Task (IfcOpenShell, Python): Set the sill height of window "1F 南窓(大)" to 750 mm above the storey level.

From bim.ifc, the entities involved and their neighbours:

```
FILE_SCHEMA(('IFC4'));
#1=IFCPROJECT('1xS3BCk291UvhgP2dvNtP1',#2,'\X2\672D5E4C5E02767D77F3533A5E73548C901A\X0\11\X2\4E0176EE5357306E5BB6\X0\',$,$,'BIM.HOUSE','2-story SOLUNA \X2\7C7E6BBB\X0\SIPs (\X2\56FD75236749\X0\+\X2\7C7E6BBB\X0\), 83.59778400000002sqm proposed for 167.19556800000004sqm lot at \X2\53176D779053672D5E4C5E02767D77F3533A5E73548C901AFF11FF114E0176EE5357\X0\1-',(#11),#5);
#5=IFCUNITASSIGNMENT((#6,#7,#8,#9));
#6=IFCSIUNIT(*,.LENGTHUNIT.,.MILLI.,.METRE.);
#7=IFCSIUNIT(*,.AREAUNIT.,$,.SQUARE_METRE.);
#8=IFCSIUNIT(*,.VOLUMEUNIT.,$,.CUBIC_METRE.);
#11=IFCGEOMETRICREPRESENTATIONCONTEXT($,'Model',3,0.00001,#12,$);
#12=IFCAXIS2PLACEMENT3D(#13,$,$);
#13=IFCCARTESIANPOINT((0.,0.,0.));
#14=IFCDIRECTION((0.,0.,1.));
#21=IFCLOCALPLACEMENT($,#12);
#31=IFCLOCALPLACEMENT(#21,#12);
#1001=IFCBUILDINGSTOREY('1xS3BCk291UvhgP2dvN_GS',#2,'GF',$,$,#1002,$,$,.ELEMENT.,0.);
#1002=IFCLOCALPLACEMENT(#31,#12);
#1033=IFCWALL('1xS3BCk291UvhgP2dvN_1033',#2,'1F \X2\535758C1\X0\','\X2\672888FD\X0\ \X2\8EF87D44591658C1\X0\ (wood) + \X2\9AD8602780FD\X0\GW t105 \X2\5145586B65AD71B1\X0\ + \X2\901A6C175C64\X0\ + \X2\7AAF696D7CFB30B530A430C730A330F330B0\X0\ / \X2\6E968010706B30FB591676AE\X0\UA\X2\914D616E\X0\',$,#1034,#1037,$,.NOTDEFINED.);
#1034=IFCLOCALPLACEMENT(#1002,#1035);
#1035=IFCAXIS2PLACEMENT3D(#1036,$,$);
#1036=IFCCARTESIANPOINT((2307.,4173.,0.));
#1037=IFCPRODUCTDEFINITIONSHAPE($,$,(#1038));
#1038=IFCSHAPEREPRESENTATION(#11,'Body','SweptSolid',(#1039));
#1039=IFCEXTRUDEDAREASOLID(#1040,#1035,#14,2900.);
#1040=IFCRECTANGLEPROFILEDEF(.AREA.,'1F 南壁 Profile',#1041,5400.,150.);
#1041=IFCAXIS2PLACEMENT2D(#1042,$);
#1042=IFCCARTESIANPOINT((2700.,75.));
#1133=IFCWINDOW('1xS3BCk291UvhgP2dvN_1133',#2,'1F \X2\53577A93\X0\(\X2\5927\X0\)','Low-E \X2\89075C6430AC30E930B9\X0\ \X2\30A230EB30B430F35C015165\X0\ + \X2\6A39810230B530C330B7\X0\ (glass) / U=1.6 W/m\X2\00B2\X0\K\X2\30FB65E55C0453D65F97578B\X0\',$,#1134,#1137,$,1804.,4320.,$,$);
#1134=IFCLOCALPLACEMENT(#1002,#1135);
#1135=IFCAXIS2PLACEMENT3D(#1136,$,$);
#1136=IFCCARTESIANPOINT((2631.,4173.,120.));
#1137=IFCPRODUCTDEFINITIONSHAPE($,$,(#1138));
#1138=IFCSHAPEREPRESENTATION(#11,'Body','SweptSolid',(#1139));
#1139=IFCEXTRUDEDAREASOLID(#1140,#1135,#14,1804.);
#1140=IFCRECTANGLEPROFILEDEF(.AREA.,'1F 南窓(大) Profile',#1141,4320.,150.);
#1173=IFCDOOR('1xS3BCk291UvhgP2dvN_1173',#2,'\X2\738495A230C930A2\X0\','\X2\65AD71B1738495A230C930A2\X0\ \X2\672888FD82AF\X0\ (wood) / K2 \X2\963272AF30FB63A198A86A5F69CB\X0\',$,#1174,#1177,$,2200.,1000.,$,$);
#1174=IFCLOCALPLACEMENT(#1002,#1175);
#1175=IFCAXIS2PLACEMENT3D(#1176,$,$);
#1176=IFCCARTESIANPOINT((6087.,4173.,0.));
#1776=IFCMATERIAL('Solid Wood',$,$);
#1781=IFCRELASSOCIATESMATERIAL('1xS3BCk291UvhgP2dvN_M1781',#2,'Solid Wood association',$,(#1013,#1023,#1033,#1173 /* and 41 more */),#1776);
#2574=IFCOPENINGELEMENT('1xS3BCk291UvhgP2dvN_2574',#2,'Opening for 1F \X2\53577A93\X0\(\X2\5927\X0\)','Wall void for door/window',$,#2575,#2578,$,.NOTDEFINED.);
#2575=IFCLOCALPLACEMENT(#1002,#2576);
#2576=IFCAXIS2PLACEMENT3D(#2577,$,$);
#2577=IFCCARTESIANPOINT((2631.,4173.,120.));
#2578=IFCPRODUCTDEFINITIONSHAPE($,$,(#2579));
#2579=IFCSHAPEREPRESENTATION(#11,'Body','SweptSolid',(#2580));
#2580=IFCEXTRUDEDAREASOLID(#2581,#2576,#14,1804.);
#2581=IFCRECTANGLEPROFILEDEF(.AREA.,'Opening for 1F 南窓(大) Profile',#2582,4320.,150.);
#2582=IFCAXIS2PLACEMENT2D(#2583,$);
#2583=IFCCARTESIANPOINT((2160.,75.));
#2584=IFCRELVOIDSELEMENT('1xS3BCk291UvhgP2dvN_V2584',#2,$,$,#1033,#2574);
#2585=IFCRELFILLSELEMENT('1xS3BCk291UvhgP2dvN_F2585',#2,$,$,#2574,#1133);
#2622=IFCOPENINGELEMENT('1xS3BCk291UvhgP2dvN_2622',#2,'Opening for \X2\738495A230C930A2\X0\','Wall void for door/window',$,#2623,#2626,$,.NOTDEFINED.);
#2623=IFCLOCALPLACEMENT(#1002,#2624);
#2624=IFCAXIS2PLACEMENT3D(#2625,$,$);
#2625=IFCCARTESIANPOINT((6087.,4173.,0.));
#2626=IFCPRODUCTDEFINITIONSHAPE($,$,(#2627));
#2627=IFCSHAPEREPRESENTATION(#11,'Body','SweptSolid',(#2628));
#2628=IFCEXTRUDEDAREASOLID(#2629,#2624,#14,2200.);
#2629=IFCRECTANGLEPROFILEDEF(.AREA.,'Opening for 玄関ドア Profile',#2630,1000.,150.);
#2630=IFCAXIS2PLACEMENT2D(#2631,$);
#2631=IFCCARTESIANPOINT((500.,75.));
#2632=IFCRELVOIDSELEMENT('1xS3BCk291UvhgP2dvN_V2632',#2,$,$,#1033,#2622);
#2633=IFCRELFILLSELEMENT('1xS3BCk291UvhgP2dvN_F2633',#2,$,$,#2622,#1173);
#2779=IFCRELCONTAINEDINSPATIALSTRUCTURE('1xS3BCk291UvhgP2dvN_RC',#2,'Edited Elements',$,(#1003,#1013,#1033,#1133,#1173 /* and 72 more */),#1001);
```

```python
import numpy as np
import ifcopenshell
import ifcopenshell.api.geometry
import ifcopenshell.geom
import ifcopenshell.util.element
import ifcopenshell.util.placement
import ifcopenshell.util.shape
import ifcopenshell.util.unit

model = ifcopenshell.open("bim.ifc")
unit_scale = ifcopenshell.util.unit.calculate_unit_scale(model)

window = model.by_guid("1xS3BCk291UvhgP2dvN_1133")
opening = window.FillsVoids[0].RelatingOpeningElement
storey = ifcopenshell.util.element.get_container(window, ifc_class="IfcBuildingStorey")
level = ifcopenshell.util.placement.get_local_placement(storey.ObjectPlacement)[2, 3]

# The opening's origin need not be at the sill, so measure its lowest point.
shape = ifcopenshell.geom.create_shape(ifcopenshell.geom.settings(), opening)
bottom = ifcopenshell.util.shape.get_shape_bottom_elevation(shape, shape.geometry) / unit_scale
dz = level + 0.75 / unit_scale - bottom

shift = np.array([0.0, 0.0, dz])
# The window is not placed relative to its opening, so move both.
for product in (opening, window):
    matrix = ifcopenshell.util.placement.get_local_placement(product.ObjectPlacement)
    matrix[:3, 3] += shift
    ifcopenshell.api.geometry.edit_object_placement(model, product=product, matrix=matrix, is_si=False)

print(f"moved by {dz * unit_scale:+.3f} m")

model.write("bim_updated.ifc")
```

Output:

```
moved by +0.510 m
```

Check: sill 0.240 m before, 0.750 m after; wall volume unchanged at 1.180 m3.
